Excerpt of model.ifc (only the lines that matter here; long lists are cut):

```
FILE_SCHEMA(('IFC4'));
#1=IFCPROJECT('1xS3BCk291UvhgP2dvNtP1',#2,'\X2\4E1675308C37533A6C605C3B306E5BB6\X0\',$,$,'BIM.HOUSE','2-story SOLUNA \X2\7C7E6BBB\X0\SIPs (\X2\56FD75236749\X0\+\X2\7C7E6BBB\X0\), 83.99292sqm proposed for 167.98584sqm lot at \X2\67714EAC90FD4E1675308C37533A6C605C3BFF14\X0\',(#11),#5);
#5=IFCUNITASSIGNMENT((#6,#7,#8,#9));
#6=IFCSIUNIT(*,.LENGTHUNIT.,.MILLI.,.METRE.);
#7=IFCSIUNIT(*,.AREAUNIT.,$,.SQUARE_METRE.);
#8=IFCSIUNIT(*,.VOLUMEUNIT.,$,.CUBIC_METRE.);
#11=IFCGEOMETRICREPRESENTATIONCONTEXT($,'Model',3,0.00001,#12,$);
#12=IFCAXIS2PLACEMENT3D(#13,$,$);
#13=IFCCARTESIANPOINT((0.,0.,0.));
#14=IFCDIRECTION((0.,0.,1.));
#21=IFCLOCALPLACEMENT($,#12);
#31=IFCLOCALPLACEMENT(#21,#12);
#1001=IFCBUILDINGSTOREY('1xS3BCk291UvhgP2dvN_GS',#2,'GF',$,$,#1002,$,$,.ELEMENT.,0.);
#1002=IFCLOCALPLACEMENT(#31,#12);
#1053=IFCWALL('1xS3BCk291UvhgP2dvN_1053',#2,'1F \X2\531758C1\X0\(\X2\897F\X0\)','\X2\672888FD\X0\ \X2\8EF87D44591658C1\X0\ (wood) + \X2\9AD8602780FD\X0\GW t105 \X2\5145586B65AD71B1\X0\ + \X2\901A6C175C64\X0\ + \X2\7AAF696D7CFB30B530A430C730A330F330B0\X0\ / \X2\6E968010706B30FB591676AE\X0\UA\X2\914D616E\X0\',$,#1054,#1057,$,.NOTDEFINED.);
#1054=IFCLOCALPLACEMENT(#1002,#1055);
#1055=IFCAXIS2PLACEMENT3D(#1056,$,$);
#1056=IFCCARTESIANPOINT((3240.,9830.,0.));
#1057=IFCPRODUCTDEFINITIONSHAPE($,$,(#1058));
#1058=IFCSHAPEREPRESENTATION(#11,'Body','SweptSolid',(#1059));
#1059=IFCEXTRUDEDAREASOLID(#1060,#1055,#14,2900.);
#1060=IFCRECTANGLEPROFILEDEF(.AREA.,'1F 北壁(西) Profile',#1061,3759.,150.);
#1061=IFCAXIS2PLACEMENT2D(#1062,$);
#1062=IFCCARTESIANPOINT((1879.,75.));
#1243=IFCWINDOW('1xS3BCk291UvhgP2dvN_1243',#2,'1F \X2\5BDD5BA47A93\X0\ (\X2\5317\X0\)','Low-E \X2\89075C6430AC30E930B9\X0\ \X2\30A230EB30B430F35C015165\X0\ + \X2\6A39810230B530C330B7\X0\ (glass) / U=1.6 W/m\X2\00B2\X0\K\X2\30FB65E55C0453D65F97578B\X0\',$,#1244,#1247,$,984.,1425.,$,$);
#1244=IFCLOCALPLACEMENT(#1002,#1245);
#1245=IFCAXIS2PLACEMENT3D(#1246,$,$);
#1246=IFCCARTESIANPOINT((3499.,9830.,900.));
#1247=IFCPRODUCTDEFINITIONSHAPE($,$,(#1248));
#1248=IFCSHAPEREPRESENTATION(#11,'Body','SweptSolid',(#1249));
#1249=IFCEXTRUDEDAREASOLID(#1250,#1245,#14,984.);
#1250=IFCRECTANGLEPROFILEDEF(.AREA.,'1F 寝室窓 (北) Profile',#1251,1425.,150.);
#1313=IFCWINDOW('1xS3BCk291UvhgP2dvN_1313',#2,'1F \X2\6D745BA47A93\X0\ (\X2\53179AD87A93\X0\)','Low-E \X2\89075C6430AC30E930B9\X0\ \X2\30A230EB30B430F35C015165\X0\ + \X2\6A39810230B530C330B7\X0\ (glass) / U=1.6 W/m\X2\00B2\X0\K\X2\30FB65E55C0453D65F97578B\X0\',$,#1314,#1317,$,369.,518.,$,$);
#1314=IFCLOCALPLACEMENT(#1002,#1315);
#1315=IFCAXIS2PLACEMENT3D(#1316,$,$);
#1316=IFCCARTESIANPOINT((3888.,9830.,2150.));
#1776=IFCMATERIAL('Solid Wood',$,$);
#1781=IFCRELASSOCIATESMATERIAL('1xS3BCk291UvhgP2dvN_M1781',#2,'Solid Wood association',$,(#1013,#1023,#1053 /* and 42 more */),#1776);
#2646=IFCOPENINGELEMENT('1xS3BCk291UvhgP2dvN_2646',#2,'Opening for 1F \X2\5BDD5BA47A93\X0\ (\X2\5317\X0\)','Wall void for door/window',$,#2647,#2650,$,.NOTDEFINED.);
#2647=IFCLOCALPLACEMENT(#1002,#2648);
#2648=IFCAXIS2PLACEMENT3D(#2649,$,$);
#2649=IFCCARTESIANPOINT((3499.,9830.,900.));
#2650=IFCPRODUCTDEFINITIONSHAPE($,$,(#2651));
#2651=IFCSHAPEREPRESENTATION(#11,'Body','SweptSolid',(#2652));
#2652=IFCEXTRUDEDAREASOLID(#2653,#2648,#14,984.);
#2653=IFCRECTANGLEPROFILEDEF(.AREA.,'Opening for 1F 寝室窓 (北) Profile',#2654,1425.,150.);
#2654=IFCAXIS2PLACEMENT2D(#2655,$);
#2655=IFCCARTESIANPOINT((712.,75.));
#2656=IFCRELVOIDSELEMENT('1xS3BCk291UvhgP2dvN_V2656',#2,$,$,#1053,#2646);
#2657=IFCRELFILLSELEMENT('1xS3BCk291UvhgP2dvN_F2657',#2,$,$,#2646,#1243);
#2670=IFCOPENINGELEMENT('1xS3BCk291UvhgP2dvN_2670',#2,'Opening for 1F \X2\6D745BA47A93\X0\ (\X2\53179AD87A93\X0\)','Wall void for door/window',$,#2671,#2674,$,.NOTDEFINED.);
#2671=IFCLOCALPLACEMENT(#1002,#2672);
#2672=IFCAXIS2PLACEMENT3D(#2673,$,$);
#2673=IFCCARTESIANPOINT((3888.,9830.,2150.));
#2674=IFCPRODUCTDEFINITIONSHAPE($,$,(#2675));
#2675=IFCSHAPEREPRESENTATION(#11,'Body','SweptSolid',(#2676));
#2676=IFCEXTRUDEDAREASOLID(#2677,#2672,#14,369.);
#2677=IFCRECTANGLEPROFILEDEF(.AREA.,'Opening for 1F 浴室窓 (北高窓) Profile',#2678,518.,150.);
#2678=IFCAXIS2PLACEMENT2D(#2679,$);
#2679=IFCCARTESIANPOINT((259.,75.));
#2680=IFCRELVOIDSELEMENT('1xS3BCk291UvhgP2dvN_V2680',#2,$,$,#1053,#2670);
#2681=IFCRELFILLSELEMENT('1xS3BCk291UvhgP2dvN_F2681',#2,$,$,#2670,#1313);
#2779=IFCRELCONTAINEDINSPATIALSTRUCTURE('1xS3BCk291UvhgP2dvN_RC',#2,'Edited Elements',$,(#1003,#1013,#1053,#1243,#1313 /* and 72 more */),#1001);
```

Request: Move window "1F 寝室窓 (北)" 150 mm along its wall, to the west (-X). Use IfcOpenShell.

```python
import ifcopenshell
import ifcopenshell.api.geometry
import ifcopenshell.util.placement
import ifcopenshell.util.unit

model = ifcopenshell.open("model.ifc")
unit_scale = ifcopenshell.util.unit.calculate_unit_scale(model)

window = model.by_guid("1xS3BCk291UvhgP2dvN_1243")
opening = window.FillsVoids[0].RelatingOpeningElement
wall = opening.VoidsElements[0].RelatingBuildingElement

wall_matrix = ifcopenshell.util.placement.get_local_placement(wall.ObjectPlacement)
shift = wall_matrix[:3, 0] * -0.15 / unit_scale
before = ifcopenshell.util.placement.get_local_placement(window.ObjectPlacement)[:3, 3].copy()

# The window is not placed relative to its opening, so move both.
for product in (opening, window):
    matrix = ifcopenshell.util.placement.get_local_placement(product.ObjectPlacement)
    matrix[:3, 3] += shift
    ifcopenshell.api.geometry.edit_object_placement(model, product=product, matrix=matrix, is_si=False)

after = ifcopenshell.util.placement.get_local_placement(window.ObjectPlacement)[:3, 3]
print("window moved by", (after - before).round(3) + 0.0)

model.write("model-out.ifc")
```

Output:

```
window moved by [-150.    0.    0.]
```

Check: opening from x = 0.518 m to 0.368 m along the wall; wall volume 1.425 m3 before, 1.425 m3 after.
